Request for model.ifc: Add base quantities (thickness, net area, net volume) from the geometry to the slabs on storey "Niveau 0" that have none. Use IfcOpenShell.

First a look at what the model holds.

```python
import ifcopenshell
import ifcopenshell.util.element
import ifcopenshell.util.unit

model = ifcopenshell.open("model.ifc")
print(model.schema)
for unit_type in ("LENGTHUNIT", "AREAUNIT", "VOLUMEUNIT"):
    print(unit_type, ifcopenshell.util.unit.calculate_unit_scale(model, unit_type))
storey = next(s for s in model.by_type("IfcBuildingStorey") if s.Name == "Niveau 0")
slabs = [e for e in ifcopenshell.util.element.get_decomposition(storey) if e.is_a("IfcSlab")]
for e in sorted(slabs, key=lambda e: e.id()):
    print(e.id(), e.is_a(), e.Name, list(ifcopenshell.util.element.get_psets(e, qtos_only=True)), sep=" | ")
```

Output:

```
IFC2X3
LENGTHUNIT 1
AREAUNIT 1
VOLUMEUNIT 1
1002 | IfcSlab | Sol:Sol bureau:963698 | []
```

```python
import ifcopenshell
import ifcopenshell.api.pset
import ifcopenshell.geom
import ifcopenshell.util.element
import ifcopenshell.util.shape
import ifcopenshell.util.unit

model = ifcopenshell.open("model.ifc")
unit_scale = ifcopenshell.util.unit.calculate_unit_scale(model)
area_scale = ifcopenshell.util.unit.calculate_unit_scale(model, "AREAUNIT")
volume_scale = ifcopenshell.util.unit.calculate_unit_scale(model, "VOLUMEUNIT")
settings = ifcopenshell.geom.settings()

storey = next(s for s in model.by_type("IfcBuildingStorey") if s.Name == "Niveau 0")
slabs = [e for e in ifcopenshell.util.element.get_decomposition(storey) if e.is_a("IfcSlab")]

for e in sorted(slabs, key=lambda e: e.id()):
    if ifcopenshell.util.element.get_psets(e, qtos_only=True, should_inherit=False):
        continue
    # Geometry comes back in metres, in the element's own axes.
    shape = ifcopenshell.geom.create_shape(settings, e)
    values = {
        "Width": ifcopenshell.util.shape.get_z(shape.geometry) / unit_scale,
        "NetArea": ifcopenshell.util.shape.get_footprint_area(shape.geometry) / area_scale,
        "NetVolume": ifcopenshell.util.shape.get_volume(shape.geometry) / volume_scale,
    }
    qto = ifcopenshell.api.pset.add_qto(model, product=e, name="BaseQuantities")
    ifcopenshell.api.pset.edit_qto(model, qto=qto, properties=values)
    print(e.id(), {k: round(v, 3) for k, v in values.items()})

model.write("model_edited.ifc")
```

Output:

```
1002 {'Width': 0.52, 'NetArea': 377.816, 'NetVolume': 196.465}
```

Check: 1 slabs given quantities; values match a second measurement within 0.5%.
